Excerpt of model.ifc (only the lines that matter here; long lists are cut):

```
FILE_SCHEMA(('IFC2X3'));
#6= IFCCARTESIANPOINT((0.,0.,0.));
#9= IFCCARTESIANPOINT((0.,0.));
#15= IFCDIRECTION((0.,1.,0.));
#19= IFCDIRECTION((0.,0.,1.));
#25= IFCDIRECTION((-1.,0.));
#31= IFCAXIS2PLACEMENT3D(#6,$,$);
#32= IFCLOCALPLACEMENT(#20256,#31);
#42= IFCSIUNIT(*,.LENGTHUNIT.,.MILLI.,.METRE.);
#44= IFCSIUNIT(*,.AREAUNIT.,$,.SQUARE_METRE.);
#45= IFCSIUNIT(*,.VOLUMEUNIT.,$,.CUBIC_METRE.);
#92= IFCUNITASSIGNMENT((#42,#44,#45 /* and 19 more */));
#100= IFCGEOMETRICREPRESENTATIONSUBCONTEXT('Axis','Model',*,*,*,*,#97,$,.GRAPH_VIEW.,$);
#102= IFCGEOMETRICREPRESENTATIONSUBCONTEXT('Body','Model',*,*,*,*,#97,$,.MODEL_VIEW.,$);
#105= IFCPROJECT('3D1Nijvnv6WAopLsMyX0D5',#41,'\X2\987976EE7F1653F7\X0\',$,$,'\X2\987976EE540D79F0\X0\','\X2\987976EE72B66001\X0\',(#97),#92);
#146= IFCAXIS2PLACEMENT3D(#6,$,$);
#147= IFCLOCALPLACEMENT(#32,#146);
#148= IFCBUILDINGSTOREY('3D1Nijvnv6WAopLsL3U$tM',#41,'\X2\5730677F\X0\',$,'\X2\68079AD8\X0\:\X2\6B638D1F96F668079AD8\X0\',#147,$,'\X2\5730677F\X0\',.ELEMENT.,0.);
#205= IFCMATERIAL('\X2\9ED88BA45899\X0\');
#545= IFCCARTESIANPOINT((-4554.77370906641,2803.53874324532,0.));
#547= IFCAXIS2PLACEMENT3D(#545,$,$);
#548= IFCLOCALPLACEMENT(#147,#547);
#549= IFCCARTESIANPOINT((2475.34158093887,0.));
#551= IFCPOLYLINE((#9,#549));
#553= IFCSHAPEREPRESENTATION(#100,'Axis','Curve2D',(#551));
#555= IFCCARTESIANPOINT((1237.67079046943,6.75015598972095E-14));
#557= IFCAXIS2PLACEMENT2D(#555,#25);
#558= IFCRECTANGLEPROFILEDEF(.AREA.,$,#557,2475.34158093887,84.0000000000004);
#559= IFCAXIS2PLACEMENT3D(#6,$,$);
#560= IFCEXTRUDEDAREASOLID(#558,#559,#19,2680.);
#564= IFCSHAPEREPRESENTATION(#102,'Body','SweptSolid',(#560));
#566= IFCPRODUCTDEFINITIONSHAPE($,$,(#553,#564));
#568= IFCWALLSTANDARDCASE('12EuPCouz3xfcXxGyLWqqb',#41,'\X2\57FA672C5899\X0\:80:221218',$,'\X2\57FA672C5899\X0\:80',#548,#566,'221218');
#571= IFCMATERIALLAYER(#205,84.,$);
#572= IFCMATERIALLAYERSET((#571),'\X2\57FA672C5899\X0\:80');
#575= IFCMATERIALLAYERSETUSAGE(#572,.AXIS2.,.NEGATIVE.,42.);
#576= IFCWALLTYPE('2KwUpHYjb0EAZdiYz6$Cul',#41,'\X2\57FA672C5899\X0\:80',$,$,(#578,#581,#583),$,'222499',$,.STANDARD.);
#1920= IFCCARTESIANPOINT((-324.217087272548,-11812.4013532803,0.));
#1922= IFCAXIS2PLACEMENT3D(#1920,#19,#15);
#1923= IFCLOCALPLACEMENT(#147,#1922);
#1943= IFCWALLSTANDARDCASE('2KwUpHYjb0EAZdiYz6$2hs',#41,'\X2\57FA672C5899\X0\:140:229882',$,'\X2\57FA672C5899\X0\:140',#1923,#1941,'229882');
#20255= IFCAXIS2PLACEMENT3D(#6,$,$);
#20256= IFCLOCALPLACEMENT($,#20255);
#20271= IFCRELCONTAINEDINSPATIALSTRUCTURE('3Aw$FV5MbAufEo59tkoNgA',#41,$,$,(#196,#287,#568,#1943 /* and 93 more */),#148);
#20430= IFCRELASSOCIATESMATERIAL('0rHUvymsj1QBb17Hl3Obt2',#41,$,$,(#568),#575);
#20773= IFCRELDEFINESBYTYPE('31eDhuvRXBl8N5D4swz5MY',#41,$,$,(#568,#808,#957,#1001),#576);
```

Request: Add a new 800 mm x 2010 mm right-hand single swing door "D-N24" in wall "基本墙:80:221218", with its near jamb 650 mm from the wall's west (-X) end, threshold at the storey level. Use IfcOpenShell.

```python
import numpy as np
import ifcopenshell
import ifcopenshell.api.feature
import ifcopenshell.api.geometry
import ifcopenshell.api.root
import ifcopenshell.api.spatial
import ifcopenshell.api.type
import ifcopenshell.geom
import ifcopenshell.util.element
import ifcopenshell.util.placement
import ifcopenshell.util.representation
import ifcopenshell.util.shape
import ifcopenshell.util.unit

model = ifcopenshell.open("model.ifc")
unit_scale = ifcopenshell.util.unit.calculate_unit_scale(model)
settings = ifcopenshell.geom.settings()


def volume(element):
    """Net volume in cubic metres, openings subtracted."""
    shape = ifcopenshell.geom.create_shape(settings, element)
    return ifcopenshell.util.shape.get_volume(shape.geometry)


wall = model.by_guid("12EuPCouz3xfcXxGyLWqqb")
storey = ifcopenshell.util.element.get_container(wall, ifc_class="IfcBuildingStorey")
context = ifcopenshell.util.representation.get_context(model, "Model", "Body", "MODEL_VIEW")
before = volume(wall)

width, height, from_end, sill = 0.8, 2.01, 0.65, 0.0  # metres

# The wall runs along its own X axis, and the end named is its -X end.
wall_shape = ifcopenshell.geom.create_shape(settings, wall)
x, y, z = ifcopenshell.util.shape.get_vertices(wall_shape.geometry).T
start = x.min() + from_end
face, thickness = float(y.min()), float(y.max() - y.min())
wall_matrix = ifcopenshell.util.placement.get_local_placement(wall.ObjectPlacement)
level = ifcopenshell.util.placement.get_local_placement(storey.ObjectPlacement)[2, 3]


def in_wall(x, y):
    """Placement at x, y metres in the wall's axes, at sill height."""
    matrix = wall_matrix.copy()
    matrix[:, 3] = wall_matrix @ np.array([x / unit_scale, y / unit_scale, 0.0, 1.0])
    matrix[2, 3] = level + sill / unit_scale
    return matrix


# Opening: a box that overshoots both wall faces by 50 mm.
opening = ifcopenshell.api.root.create_entity(model, ifc_class="IfcOpeningElement")
box = ifcopenshell.api.geometry.add_wall_representation(
    model, context=context, length=width, height=height, thickness=thickness + 0.1
)
ifcopenshell.api.geometry.assign_representation(model, product=opening, representation=box)
ifcopenshell.api.geometry.edit_object_placement(model, product=opening, matrix=in_wall(start, face - 0.05), is_si=False)
ifcopenshell.api.feature.add_feature(model, feature=opening, element=wall)

door = ifcopenshell.api.root.create_entity(model, ifc_class="IfcDoor", name="D-N24")
door.OverallWidth, door.OverallHeight = width / unit_scale, height / unit_scale
body = ifcopenshell.api.geometry.add_door_representation(
    model,
    context=context,
    overall_width=door.OverallWidth,
    overall_height=door.OverallHeight,
    operation_type="SINGLE_SWING_RIGHT",
    lining_properties={"LiningDepth": thickness / unit_scale, "ThresholdDepth": thickness / unit_scale},
)
ifcopenshell.api.geometry.assign_representation(model, product=door, representation=body)
ifcopenshell.api.spatial.assign_container(model, products=[door], relating_structure=storey)
fills = ifcopenshell.api.feature.add_filling(model, opening=opening, element=door)
fills.OwnerHistory = door.OwnerHistory  # required in IFC2X3

# IFC2X3 keeps the operation on the door style.
style = ifcopenshell.api.root.create_entity(model, ifc_class="IfcDoorStyle", name="D-N24")
style.OperationType, style.ConstructionType = "SINGLE_SWING_RIGHT", "NOTDEFINED"
style.ParameterTakesPrecedence = style.Sizeable = False
ifcopenshell.api.type.assign_type(model, related_objects=[door], relating_type=style)

# The lining spans the wall, so the door starts at the wall face.
ifcopenshell.api.geometry.edit_object_placement(model, product=door, matrix=in_wall(start, face), is_si=False)

after = volume(wall)

print(f"wall volume {before:.3f} -> {after:.3f} m3")

model.write("model_edited.ifc")
```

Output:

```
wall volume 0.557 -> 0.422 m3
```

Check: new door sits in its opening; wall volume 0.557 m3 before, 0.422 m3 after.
